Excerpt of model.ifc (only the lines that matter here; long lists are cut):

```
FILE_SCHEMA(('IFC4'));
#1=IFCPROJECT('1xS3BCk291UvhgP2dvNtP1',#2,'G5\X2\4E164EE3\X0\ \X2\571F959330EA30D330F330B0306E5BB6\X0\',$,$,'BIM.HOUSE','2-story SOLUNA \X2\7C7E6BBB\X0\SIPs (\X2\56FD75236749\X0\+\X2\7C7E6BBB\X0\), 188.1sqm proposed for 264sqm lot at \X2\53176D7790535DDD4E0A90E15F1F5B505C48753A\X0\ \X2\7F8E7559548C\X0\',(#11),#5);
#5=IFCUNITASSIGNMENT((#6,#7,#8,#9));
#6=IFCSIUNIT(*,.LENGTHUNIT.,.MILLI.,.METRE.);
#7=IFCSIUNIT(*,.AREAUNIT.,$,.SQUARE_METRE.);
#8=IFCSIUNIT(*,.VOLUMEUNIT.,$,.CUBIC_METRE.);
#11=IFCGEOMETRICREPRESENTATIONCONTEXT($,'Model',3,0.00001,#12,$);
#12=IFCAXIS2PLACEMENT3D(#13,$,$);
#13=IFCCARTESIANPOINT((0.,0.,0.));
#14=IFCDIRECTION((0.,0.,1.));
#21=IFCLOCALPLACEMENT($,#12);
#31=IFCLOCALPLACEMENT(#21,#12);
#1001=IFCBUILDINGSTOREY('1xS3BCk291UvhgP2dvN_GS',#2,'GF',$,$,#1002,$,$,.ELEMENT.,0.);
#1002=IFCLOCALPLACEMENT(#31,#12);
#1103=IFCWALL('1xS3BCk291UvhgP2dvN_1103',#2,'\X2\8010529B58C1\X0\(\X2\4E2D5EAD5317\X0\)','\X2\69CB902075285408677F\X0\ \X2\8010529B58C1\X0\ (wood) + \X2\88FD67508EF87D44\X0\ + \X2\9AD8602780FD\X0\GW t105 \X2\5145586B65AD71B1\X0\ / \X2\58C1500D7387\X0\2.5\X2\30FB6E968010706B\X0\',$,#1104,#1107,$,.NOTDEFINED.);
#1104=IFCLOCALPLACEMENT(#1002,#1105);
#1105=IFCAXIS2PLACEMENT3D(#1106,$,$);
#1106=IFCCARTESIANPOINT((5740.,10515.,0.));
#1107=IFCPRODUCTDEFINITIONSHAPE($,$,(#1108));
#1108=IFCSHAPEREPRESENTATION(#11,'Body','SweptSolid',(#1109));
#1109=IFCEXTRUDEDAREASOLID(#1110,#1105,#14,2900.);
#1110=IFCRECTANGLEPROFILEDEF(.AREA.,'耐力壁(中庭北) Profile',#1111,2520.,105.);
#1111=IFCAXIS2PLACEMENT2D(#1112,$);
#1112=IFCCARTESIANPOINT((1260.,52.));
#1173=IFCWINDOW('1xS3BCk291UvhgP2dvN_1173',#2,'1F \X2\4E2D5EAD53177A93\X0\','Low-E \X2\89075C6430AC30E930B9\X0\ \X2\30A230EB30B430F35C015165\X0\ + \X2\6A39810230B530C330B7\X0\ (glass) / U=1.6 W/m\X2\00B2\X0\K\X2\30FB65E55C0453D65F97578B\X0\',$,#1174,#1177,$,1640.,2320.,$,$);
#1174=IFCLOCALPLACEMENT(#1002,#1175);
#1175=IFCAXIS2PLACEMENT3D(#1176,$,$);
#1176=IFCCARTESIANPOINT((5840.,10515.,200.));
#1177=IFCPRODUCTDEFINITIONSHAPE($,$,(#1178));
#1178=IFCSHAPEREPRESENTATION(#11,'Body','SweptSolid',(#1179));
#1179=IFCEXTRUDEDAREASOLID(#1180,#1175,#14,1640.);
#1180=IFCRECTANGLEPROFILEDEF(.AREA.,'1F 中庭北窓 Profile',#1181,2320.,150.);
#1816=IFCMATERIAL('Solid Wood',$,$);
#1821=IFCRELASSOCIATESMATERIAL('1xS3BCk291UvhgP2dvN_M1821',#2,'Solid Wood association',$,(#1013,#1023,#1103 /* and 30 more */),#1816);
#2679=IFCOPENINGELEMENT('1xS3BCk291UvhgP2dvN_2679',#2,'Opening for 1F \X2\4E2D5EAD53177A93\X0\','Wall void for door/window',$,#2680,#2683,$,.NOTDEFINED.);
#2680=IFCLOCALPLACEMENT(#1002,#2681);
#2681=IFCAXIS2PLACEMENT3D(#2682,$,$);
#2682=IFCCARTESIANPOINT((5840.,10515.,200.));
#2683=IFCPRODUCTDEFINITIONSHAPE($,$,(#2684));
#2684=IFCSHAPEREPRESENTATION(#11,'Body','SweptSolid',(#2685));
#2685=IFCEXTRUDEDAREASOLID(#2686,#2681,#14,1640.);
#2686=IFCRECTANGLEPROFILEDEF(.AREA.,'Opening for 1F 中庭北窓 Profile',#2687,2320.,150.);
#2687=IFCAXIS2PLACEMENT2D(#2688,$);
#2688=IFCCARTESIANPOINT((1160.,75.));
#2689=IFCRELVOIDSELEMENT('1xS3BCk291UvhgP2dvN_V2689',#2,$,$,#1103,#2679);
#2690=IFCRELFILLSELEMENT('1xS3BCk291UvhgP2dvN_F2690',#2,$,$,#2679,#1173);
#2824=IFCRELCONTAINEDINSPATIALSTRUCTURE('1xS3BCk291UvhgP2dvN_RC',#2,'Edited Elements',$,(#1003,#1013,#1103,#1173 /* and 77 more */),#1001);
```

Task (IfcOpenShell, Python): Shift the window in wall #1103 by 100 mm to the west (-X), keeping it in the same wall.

```python
import ifcopenshell
import ifcopenshell.api.geometry
import ifcopenshell.util.placement

model = ifcopenshell.open("model.ifc")

window = model.by_guid("1xS3BCk291UvhgP2dvN_1173")
opening = window.FillsVoids[0].RelatingOpeningElement
wall = opening.VoidsElements[0].RelatingBuildingElement

wall_matrix = ifcopenshell.util.placement.get_local_placement(wall.ObjectPlacement)
shift = wall_matrix[:3, 0] * -100.0
before = ifcopenshell.util.placement.get_local_placement(window.ObjectPlacement)[:3, 3].copy()

# The window is not placed relative to its opening, so move both.
for product in (opening, window):
    matrix = ifcopenshell.util.placement.get_local_placement(product.ObjectPlacement)
    matrix[:3, 3] += shift
    ifcopenshell.api.geometry.edit_object_placement(model, product=product, matrix=matrix, is_si=False)

after = ifcopenshell.util.placement.get_local_placement(window.ObjectPlacement)[:3, 3]
print("window moved by", (after - before).round(3) + 0.0)

model.write("model_updated.ifc")
```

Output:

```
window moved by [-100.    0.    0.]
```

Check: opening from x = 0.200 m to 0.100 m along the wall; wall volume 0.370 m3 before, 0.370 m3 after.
